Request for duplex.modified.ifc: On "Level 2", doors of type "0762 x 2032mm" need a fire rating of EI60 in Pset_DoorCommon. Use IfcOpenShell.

First a look at what the model holds.

```python
import ifcopenshell
import ifcopenshell.util.element

model = ifcopenshell.open("duplex.modified.ifc")
print(model.schema)
storey = next(s for s in model.by_type("IfcBuildingStorey") if s.Name == "Level 2")
doors = [e for e in ifcopenshell.util.element.get_decomposition(storey) if e.is_a("IfcDoor")]
seen = {}
for e in doors:
    element_type = ifcopenshell.util.element.get_type(e)
    key = (element_type.Name if element_type != e and element_type else None, ifcopenshell.util.element.get_pset(e, "Pset_DoorCommon", "FireRating"))
    seen[key] = seen.get(key, 0) + 1
for (name, value), count in sorted(seen.items(), key=str):
    print(count, "x", name, "|", value)
```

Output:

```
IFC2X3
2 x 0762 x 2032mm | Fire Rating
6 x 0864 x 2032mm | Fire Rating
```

```python
import ifcopenshell
import ifcopenshell.api.pset
import ifcopenshell.util.element

model = ifcopenshell.open("duplex.modified.ifc")

storey = next(s for s in model.by_type("IfcBuildingStorey") if s.Name == "Level 2")
doors = [e for e in ifcopenshell.util.element.get_decomposition(storey) if e.is_a("IfcDoor")]

count = 0
for e in doors:
    element_type = ifcopenshell.util.element.get_type(e)
    if element_type in (None, e) or element_type.Name != "0762 x 2032mm":
        continue
    # add_pset returns the element's existing set when there is one.
    pset = ifcopenshell.api.pset.add_pset(model, product=e, name="Pset_DoorCommon")
    ifcopenshell.api.pset.edit_pset(model, pset=pset, properties={"FireRating": "EI60"})
    count += 1

print(count, "doors updated")

model.write("duplex.modified_rev.ifc")
```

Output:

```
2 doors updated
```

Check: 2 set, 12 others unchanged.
